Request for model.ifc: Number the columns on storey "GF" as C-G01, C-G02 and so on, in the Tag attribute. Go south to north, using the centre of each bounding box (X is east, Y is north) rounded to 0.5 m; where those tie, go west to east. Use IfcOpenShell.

First a look at what the model holds.

```python
import ifcopenshell
import ifcopenshell.util.element
import ifcopenshell.util.placement

model = ifcopenshell.open("model.ifc")
print(model.schema)
storey = next(s for s in model.by_type("IfcBuildingStorey") if s.Name == "GF")
columns = [e for e in ifcopenshell.util.element.get_decomposition(storey) if e.is_a("IfcColumn")]
for e in sorted(columns, key=lambda e: e.id()):
    origin = ifcopenshell.util.placement.get_local_placement(e.ObjectPlacement)[:3, 3]
    print(e.id(), e.Tag, e.Name, origin.round(2) + 0.0, sep=" | ")
```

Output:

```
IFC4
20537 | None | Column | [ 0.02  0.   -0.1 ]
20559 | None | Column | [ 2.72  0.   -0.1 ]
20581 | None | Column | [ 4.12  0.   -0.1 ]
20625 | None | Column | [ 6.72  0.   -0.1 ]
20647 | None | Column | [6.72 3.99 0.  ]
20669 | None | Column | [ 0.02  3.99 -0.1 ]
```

```python
import ifcopenshell
import ifcopenshell.geom
import ifcopenshell.util.element
import ifcopenshell.util.shape

model = ifcopenshell.open("model.ifc")
settings = ifcopenshell.geom.settings()
settings.set("use-world-coords", True)


def centre(element):
    shape = ifcopenshell.geom.create_shape(settings, element)
    return ifcopenshell.util.shape.get_bbox_centroid(shape.geometry)


storey = next(s for s in model.by_type("IfcBuildingStorey") if s.Name == "GF")
columns = [e for e in ifcopenshell.util.element.get_decomposition(storey) if e.is_a("IfcColumn")]

# Insertion points can sit at a corner or the storey origin, so sort by the geometry (in metres).
centres = {e: centre(e) for e in columns}
columns.sort(key=lambda e: (round(centres[e][1] / 0.5), centres[e][0]))

for i, e in enumerate(columns, start=1):
    number = f"C-G{i:02d}"
    e.Tag = number
    print(e.id(), number)

model.write("model_rev.ifc")
```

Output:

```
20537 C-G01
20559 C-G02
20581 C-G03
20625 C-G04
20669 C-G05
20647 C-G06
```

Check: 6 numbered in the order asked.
